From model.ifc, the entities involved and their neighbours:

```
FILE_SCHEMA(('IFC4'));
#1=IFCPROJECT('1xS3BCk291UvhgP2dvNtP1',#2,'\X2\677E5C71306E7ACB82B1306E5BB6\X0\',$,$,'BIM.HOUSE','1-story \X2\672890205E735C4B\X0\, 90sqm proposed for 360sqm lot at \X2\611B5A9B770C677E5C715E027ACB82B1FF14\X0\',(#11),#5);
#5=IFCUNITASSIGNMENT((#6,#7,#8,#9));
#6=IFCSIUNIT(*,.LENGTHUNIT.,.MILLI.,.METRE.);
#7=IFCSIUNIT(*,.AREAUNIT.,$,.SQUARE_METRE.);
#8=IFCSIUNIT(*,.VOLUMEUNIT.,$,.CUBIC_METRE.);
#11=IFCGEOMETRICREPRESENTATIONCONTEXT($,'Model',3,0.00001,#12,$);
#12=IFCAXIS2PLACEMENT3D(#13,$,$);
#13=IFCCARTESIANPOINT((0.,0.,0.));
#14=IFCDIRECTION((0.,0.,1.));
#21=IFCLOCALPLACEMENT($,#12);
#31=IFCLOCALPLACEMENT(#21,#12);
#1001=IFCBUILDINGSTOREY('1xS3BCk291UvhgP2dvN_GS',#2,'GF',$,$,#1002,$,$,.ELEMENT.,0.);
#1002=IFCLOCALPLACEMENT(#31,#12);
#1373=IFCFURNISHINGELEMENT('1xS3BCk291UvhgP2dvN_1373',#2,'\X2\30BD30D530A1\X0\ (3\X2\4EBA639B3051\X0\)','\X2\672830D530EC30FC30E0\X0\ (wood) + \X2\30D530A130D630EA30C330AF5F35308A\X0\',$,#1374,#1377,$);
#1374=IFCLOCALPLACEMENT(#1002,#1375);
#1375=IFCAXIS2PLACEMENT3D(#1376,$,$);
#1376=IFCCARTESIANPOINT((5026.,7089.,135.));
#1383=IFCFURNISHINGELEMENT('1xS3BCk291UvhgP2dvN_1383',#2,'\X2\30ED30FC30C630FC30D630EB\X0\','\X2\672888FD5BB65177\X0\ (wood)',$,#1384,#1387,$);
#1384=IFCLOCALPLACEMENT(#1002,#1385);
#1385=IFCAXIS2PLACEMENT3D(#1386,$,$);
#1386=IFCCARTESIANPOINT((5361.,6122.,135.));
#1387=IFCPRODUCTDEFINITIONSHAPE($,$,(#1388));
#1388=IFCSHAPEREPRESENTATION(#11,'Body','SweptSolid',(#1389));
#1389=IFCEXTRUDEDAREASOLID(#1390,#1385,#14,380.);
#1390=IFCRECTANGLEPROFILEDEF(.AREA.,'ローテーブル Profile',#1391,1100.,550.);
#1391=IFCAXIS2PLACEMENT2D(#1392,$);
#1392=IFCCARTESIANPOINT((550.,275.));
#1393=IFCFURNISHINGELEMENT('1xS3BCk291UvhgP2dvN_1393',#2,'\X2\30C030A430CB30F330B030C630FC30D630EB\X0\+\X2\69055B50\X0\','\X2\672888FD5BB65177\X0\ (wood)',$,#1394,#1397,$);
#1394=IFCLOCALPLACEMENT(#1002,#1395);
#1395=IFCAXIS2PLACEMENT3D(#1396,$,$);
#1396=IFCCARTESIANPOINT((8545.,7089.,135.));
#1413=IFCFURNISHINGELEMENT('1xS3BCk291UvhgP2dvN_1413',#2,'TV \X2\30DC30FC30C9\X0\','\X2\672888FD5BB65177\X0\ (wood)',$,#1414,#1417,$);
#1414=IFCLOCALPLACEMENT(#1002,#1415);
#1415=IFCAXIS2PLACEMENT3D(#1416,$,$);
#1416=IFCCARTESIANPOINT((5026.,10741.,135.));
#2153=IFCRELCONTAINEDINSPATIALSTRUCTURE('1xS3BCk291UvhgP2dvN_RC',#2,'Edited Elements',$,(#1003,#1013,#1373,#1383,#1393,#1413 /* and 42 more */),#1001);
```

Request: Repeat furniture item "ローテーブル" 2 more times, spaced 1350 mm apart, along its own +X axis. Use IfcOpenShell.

```python
import ifcopenshell
import ifcopenshell.api.geometry
import ifcopenshell.api.root
import ifcopenshell.util.element
import ifcopenshell.util.placement

model = ifcopenshell.open("model.ifc")


def reuse_history(source, copy):
    """copy_class also copies each property set's owner history, people and application; keep the originals."""
    for rel in copy.IsDefinedBy:
        if rel.is_a("IfcRelDefinesByProperties") and (history := rel.RelatingPropertyDefinition.OwnerHistory):
            rel.RelatingPropertyDefinition.OwnerHistory = source.OwnerHistory
            ifcopenshell.util.element.remove_deep2(model, history)


source = model.by_guid("1xS3BCk291UvhgP2dvN_1383")
base = ifcopenshell.util.placement.get_local_placement(source.ObjectPlacement)
step = base[:3, 0] * 1350.0

for i in range(1, 3):
    copy = ifcopenshell.api.root.copy_class(model, product=source)
    copy.Representation = ifcopenshell.util.element.copy_deep(
        model, source.Representation, exclude=["IfcGeometricRepresentationContext", "IfcRepresentationMap"]
    )
    reuse_history(source, copy)
    matrix = base.copy()
    matrix[:3, 3] += i * step
    print("added at", matrix[:3, 3].round(3) + 0.0)
    ifcopenshell.api.geometry.edit_object_placement(model, product=copy, matrix=matrix, is_si=False)

model.write("model-out.ifc")
```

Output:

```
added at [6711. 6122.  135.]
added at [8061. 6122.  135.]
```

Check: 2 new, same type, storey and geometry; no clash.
